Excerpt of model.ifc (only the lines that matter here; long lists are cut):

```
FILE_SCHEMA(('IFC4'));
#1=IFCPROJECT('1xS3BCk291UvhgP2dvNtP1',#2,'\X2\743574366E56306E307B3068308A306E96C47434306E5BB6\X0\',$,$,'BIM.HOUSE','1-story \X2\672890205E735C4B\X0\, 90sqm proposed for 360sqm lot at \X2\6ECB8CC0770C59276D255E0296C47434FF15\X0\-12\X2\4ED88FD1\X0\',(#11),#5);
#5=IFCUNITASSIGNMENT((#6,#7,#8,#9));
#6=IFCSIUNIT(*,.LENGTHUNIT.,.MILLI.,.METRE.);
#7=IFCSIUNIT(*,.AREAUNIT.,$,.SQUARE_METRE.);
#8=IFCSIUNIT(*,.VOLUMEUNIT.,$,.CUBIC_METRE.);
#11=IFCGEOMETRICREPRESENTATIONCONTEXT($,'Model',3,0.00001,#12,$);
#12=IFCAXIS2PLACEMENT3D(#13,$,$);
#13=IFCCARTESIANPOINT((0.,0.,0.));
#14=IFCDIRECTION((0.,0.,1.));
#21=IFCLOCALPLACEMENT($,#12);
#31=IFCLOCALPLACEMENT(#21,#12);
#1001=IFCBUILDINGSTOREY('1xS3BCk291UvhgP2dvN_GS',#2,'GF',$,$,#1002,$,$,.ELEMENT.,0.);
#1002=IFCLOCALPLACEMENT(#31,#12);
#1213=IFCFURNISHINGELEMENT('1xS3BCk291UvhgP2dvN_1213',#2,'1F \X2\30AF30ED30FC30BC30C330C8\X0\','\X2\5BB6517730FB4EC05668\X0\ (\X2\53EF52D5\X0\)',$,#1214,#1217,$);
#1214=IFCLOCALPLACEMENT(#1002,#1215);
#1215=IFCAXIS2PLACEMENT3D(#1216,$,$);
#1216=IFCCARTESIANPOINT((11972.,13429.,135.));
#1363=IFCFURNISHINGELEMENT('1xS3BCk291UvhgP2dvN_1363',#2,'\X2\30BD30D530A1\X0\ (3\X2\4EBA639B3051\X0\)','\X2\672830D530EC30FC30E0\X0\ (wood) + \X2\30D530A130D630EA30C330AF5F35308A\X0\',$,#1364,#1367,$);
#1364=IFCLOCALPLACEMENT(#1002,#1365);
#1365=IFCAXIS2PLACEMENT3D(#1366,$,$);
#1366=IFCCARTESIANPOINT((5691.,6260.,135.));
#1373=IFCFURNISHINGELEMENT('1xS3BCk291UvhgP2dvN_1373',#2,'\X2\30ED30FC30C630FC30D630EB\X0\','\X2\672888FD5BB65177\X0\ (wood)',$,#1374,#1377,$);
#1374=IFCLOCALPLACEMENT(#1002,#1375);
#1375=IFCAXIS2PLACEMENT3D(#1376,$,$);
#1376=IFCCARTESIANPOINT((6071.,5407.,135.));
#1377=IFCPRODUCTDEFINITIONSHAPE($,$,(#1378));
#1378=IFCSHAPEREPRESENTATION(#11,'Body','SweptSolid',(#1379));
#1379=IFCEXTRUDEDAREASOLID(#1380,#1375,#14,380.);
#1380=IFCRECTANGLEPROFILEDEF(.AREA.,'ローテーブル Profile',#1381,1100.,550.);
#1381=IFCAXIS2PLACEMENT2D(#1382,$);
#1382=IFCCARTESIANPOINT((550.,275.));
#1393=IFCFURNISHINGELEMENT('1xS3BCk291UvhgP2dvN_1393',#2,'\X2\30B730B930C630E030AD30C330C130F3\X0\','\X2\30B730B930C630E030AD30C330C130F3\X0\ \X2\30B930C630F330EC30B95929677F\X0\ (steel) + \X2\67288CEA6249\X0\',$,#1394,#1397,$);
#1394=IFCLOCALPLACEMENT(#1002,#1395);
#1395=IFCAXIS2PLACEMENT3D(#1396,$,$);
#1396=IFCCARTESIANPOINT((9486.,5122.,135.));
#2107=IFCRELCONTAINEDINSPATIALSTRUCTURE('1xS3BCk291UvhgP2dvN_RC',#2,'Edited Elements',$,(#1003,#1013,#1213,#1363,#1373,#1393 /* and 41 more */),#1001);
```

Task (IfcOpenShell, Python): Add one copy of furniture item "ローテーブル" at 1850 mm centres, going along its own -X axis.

```python
import ifcopenshell
import ifcopenshell.api.geometry
import ifcopenshell.api.root
import ifcopenshell.util.element
import ifcopenshell.util.placement
import ifcopenshell.util.unit

model = ifcopenshell.open("model.ifc")
unit_scale = ifcopenshell.util.unit.calculate_unit_scale(model)


def reuse_history(source, copy):
    """copy_class also copies each property set's owner history, people and application; keep the originals."""
    for rel in copy.IsDefinedBy:
        if rel.is_a("IfcRelDefinesByProperties") and (history := rel.RelatingPropertyDefinition.OwnerHistory):
            rel.RelatingPropertyDefinition.OwnerHistory = source.OwnerHistory
            ifcopenshell.util.element.remove_deep2(model, history)


source = model.by_id(1373)
base = ifcopenshell.util.placement.get_local_placement(source.ObjectPlacement)
step = -base[:3, 0] * 1.85 / unit_scale

for i in range(1, 2):
    copy = ifcopenshell.api.root.copy_class(model, product=source)
    copy.Representation = ifcopenshell.util.element.copy_deep(
        model, source.Representation, exclude=["IfcGeometricRepresentationContext", "IfcRepresentationMap"]
    )
    reuse_history(source, copy)
    matrix = base.copy()
    matrix[:3, 3] += i * step
    print("added at", matrix[:3, 3].round(3) + 0.0)
    ifcopenshell.api.geometry.edit_object_placement(model, product=copy, matrix=matrix, is_si=False)

model.write("model-out.ifc")
```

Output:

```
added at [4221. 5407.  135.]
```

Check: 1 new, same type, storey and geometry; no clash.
